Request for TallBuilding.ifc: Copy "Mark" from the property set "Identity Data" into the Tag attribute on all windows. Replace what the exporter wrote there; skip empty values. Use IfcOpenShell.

First a look at what the model holds.

```python
import ifcopenshell
import ifcopenshell.util.element

model = ifcopenshell.open("TallBuilding.ifc")
print(model.schema)
windows = model.by_type("IfcWindow")
print(len(windows), "windows")
for e in windows[:8]:
    source = ifcopenshell.util.element.get_pset(e, "Identity Data", "Mark")
    target = e.Tag
    print(e.id(), repr(source), repr(target), sep=" | ")
```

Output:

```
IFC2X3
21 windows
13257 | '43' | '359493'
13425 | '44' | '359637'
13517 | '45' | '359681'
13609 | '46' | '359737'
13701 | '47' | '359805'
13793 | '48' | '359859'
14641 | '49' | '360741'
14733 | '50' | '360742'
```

```python
import ifcopenshell
import ifcopenshell.util.element

model = ifcopenshell.open("TallBuilding.ifc")

count = 0
for e in model.by_type("IfcWindow"):
    value = ifcopenshell.util.element.get_pset(e, "Identity Data", "Mark")
    current = e.Tag
    if not value or not value.strip() or current == value:
        continue
    e.Tag = value
    count += 1

print(count, "windows updated")

model.write("TallBuilding_updated.ifc")
```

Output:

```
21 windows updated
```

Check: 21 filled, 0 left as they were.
